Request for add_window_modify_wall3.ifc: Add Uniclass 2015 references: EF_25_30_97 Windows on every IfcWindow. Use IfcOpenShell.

First a look at what the model holds.

```python
import ifcopenshell

model = ifcopenshell.open("add_window_modify_wall3.ifc")
print(model.schema)
print("classifications:", [c.Name for c in model.by_type("IfcClassification")])
for ifc_class in ("IfcDoor", "IfcRoof", "IfcStair", "IfcWall", "IfcWindow"):
    print(ifc_class, len(model.by_type(ifc_class)))
```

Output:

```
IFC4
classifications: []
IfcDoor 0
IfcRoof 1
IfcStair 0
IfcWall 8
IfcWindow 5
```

```python
import ifcopenshell
import ifcopenshell.api.classification

model = ifcopenshell.open("add_window_modify_wall3.ifc")

system = ifcopenshell.api.classification.add_classification(model, classification="Uniclass 2015")

codes = {
    "IfcWindow": ("EF_25_30_97", "Windows"),
}
for ifc_class, (code, name) in codes.items():
    products = model.by_type(ifc_class)
    ifcopenshell.api.classification.add_reference(
        model, products=products, classification=system, identification=code, name=name
    )
    print(code, len(products))

model.write("add_window_modify_wall3-out.ifc")
```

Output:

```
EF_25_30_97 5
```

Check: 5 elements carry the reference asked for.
